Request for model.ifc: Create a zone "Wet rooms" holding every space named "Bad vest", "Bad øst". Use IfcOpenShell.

First a look at what the model holds.

```python
import ifcopenshell

model = ifcopenshell.open("model.ifc")
print(model.schema)
seen = {}
for space in model.by_type("IfcSpace"):
    seen[space.LongName] = seen.get(space.LongName, 0) + 1
for name, count in sorted(seen.items(), key=str):
    print(count, "x", name)
print("zones:", [z.Name for z in model.by_type("IfcZone")][:20])
```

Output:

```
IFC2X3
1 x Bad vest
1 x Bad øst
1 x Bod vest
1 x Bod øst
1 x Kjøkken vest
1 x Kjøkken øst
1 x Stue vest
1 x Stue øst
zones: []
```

```python
import ifcopenshell
import ifcopenshell.api.group
import ifcopenshell.api.root

model = ifcopenshell.open("model.ifc")

names = {"Bad vest", "Bad øst"}
spaces = [s for s in model.by_type("IfcSpace") if s.LongName in names]

zone = ifcopenshell.api.root.create_entity(model, ifc_class="IfcZone", name="Wet rooms")
ifcopenshell.api.group.assign_group(model, products=spaces, group=zone)
print(len(spaces), "spaces in", zone.Name)

model.write("model_rev.ifc")
```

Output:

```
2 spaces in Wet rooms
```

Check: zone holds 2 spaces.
